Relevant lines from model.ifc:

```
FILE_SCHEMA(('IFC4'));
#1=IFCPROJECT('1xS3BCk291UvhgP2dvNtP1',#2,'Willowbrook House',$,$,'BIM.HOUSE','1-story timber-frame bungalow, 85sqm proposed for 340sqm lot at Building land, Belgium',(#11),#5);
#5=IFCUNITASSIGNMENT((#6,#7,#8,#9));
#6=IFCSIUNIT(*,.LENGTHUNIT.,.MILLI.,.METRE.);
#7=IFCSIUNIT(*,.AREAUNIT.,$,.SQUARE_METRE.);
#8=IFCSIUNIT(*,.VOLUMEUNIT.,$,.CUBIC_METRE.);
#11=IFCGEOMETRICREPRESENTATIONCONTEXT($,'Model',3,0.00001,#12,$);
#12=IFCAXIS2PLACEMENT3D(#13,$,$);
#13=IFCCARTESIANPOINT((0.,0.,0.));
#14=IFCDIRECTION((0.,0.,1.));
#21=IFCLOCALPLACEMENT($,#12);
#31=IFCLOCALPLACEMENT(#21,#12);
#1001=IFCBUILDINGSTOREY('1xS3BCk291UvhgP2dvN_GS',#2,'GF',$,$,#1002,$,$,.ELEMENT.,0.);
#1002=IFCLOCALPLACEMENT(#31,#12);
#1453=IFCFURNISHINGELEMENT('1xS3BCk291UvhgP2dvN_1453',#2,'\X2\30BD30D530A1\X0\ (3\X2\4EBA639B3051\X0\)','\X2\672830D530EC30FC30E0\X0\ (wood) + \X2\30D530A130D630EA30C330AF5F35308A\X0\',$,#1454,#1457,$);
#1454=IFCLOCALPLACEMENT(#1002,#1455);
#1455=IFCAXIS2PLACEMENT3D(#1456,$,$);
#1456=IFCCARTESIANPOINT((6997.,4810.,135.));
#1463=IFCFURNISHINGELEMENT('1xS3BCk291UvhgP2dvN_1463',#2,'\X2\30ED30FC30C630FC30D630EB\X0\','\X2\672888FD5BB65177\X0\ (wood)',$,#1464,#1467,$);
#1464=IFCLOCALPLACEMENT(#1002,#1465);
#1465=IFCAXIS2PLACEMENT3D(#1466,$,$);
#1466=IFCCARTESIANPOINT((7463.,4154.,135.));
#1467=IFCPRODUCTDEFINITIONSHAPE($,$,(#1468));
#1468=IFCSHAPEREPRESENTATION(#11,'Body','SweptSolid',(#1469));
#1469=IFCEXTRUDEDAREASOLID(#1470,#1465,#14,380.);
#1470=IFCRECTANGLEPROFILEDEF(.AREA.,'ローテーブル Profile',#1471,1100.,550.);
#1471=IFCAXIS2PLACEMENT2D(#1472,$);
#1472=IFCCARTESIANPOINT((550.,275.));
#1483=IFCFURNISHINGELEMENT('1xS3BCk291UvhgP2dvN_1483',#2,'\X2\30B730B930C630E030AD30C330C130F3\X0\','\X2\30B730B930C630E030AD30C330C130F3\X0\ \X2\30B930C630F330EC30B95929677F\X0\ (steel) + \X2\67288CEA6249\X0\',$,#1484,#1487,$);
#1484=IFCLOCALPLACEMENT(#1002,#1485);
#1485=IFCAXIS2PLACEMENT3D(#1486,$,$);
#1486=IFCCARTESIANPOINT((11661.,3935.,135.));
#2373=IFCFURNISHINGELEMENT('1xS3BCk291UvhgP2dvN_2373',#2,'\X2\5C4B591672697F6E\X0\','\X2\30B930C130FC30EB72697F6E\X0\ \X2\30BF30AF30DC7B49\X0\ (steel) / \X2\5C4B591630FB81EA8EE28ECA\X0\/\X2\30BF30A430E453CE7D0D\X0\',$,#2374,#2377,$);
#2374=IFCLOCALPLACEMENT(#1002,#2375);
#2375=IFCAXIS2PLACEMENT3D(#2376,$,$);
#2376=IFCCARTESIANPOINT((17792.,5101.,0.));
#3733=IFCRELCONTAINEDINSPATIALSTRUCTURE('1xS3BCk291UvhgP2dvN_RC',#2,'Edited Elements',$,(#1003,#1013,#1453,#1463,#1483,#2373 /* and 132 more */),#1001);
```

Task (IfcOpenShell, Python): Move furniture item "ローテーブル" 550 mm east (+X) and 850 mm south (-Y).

```python
import ifcopenshell
import ifcopenshell.api.geometry
import ifcopenshell.util.placement
import ifcopenshell.util.unit

model = ifcopenshell.open("model.ifc")
unit_scale = ifcopenshell.util.unit.calculate_unit_scale(model)

item = model.by_id(1463)
matrix = ifcopenshell.util.placement.get_local_placement(item.ObjectPlacement)
matrix[0, 3] += 0.55 / unit_scale
matrix[1, 3] -= 0.85 / unit_scale
ifcopenshell.api.geometry.edit_object_placement(model, product=item, matrix=matrix, is_si=False)

print(ifcopenshell.util.placement.get_local_placement(item.ObjectPlacement).round(3) + 0.0)

model.write("model-out.ifc")
```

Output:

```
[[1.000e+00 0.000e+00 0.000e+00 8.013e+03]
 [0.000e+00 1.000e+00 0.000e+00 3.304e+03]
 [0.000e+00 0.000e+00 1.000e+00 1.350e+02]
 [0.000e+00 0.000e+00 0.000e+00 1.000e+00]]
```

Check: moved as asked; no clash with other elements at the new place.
